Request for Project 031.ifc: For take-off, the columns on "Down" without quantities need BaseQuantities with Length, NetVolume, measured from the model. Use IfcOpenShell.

First a look at what the model holds.

```python
import ifcopenshell
import ifcopenshell.util.element
import ifcopenshell.util.unit

model = ifcopenshell.open("Project 031.ifc")
print(model.schema)
for unit_type in ("LENGTHUNIT", "AREAUNIT", "VOLUMEUNIT"):
    print(unit_type, ifcopenshell.util.unit.calculate_unit_scale(model, unit_type))
storey = next(s for s in model.by_type("IfcBuildingStorey") if s.Name == "Down")
columns = [e for e in ifcopenshell.util.element.get_decomposition(storey) if e.is_a("IfcColumn")]
for e in sorted(columns, key=lambda e: e.id()):
    print(e.id(), e.is_a(), e.Name, list(ifcopenshell.util.element.get_psets(e, qtos_only=True)), sep=" | ")
```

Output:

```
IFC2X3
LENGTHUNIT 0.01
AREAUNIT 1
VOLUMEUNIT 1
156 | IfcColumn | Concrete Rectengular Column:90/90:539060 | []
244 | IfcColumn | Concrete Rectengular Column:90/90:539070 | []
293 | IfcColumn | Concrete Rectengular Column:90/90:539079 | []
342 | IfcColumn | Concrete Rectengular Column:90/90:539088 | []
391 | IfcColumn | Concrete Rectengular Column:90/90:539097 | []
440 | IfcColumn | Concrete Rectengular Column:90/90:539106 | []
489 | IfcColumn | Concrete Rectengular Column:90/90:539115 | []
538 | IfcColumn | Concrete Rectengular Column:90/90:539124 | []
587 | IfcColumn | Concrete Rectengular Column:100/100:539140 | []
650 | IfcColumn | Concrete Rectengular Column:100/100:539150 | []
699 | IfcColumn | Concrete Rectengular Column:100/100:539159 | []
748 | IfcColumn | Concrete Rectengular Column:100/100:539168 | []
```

```python
import ifcopenshell
import ifcopenshell.api.pset
import ifcopenshell.geom
import ifcopenshell.util.element
import ifcopenshell.util.shape
import ifcopenshell.util.unit

model = ifcopenshell.open("Project 031.ifc")
unit_scale = ifcopenshell.util.unit.calculate_unit_scale(model)
volume_scale = ifcopenshell.util.unit.calculate_unit_scale(model, "VOLUMEUNIT")
settings = ifcopenshell.geom.settings()

storey = next(s for s in model.by_type("IfcBuildingStorey") if s.Name == "Down")
columns = [e for e in ifcopenshell.util.element.get_decomposition(storey) if e.is_a("IfcColumn")]

for e in sorted(columns, key=lambda e: e.id()):
    if ifcopenshell.util.element.get_psets(e, qtos_only=True, should_inherit=False):
        continue
    # Geometry comes back in metres, in the element's own axes.
    shape = ifcopenshell.geom.create_shape(settings, e)
    values = {
        "Length": ifcopenshell.util.shape.get_z(shape.geometry) / unit_scale,
        "NetVolume": ifcopenshell.util.shape.get_volume(shape.geometry) / volume_scale,
    }
    qto = ifcopenshell.api.pset.add_qto(model, product=e, name="BaseQuantities")
    ifcopenshell.api.pset.edit_qto(model, qto=qto, properties=values)
    print(e.id(), {k: round(v, 3) for k, v in values.items()})

model.write("Project 031-out.ifc")
```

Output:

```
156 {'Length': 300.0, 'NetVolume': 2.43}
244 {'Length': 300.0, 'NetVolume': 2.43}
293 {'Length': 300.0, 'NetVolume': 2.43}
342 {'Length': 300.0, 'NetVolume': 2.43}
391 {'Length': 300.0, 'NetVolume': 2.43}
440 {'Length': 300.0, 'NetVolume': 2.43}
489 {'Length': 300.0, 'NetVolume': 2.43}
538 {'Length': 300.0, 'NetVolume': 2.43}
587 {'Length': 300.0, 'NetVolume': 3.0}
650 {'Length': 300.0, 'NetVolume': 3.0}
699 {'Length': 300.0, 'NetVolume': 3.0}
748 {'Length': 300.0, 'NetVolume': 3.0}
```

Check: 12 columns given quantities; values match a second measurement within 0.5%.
